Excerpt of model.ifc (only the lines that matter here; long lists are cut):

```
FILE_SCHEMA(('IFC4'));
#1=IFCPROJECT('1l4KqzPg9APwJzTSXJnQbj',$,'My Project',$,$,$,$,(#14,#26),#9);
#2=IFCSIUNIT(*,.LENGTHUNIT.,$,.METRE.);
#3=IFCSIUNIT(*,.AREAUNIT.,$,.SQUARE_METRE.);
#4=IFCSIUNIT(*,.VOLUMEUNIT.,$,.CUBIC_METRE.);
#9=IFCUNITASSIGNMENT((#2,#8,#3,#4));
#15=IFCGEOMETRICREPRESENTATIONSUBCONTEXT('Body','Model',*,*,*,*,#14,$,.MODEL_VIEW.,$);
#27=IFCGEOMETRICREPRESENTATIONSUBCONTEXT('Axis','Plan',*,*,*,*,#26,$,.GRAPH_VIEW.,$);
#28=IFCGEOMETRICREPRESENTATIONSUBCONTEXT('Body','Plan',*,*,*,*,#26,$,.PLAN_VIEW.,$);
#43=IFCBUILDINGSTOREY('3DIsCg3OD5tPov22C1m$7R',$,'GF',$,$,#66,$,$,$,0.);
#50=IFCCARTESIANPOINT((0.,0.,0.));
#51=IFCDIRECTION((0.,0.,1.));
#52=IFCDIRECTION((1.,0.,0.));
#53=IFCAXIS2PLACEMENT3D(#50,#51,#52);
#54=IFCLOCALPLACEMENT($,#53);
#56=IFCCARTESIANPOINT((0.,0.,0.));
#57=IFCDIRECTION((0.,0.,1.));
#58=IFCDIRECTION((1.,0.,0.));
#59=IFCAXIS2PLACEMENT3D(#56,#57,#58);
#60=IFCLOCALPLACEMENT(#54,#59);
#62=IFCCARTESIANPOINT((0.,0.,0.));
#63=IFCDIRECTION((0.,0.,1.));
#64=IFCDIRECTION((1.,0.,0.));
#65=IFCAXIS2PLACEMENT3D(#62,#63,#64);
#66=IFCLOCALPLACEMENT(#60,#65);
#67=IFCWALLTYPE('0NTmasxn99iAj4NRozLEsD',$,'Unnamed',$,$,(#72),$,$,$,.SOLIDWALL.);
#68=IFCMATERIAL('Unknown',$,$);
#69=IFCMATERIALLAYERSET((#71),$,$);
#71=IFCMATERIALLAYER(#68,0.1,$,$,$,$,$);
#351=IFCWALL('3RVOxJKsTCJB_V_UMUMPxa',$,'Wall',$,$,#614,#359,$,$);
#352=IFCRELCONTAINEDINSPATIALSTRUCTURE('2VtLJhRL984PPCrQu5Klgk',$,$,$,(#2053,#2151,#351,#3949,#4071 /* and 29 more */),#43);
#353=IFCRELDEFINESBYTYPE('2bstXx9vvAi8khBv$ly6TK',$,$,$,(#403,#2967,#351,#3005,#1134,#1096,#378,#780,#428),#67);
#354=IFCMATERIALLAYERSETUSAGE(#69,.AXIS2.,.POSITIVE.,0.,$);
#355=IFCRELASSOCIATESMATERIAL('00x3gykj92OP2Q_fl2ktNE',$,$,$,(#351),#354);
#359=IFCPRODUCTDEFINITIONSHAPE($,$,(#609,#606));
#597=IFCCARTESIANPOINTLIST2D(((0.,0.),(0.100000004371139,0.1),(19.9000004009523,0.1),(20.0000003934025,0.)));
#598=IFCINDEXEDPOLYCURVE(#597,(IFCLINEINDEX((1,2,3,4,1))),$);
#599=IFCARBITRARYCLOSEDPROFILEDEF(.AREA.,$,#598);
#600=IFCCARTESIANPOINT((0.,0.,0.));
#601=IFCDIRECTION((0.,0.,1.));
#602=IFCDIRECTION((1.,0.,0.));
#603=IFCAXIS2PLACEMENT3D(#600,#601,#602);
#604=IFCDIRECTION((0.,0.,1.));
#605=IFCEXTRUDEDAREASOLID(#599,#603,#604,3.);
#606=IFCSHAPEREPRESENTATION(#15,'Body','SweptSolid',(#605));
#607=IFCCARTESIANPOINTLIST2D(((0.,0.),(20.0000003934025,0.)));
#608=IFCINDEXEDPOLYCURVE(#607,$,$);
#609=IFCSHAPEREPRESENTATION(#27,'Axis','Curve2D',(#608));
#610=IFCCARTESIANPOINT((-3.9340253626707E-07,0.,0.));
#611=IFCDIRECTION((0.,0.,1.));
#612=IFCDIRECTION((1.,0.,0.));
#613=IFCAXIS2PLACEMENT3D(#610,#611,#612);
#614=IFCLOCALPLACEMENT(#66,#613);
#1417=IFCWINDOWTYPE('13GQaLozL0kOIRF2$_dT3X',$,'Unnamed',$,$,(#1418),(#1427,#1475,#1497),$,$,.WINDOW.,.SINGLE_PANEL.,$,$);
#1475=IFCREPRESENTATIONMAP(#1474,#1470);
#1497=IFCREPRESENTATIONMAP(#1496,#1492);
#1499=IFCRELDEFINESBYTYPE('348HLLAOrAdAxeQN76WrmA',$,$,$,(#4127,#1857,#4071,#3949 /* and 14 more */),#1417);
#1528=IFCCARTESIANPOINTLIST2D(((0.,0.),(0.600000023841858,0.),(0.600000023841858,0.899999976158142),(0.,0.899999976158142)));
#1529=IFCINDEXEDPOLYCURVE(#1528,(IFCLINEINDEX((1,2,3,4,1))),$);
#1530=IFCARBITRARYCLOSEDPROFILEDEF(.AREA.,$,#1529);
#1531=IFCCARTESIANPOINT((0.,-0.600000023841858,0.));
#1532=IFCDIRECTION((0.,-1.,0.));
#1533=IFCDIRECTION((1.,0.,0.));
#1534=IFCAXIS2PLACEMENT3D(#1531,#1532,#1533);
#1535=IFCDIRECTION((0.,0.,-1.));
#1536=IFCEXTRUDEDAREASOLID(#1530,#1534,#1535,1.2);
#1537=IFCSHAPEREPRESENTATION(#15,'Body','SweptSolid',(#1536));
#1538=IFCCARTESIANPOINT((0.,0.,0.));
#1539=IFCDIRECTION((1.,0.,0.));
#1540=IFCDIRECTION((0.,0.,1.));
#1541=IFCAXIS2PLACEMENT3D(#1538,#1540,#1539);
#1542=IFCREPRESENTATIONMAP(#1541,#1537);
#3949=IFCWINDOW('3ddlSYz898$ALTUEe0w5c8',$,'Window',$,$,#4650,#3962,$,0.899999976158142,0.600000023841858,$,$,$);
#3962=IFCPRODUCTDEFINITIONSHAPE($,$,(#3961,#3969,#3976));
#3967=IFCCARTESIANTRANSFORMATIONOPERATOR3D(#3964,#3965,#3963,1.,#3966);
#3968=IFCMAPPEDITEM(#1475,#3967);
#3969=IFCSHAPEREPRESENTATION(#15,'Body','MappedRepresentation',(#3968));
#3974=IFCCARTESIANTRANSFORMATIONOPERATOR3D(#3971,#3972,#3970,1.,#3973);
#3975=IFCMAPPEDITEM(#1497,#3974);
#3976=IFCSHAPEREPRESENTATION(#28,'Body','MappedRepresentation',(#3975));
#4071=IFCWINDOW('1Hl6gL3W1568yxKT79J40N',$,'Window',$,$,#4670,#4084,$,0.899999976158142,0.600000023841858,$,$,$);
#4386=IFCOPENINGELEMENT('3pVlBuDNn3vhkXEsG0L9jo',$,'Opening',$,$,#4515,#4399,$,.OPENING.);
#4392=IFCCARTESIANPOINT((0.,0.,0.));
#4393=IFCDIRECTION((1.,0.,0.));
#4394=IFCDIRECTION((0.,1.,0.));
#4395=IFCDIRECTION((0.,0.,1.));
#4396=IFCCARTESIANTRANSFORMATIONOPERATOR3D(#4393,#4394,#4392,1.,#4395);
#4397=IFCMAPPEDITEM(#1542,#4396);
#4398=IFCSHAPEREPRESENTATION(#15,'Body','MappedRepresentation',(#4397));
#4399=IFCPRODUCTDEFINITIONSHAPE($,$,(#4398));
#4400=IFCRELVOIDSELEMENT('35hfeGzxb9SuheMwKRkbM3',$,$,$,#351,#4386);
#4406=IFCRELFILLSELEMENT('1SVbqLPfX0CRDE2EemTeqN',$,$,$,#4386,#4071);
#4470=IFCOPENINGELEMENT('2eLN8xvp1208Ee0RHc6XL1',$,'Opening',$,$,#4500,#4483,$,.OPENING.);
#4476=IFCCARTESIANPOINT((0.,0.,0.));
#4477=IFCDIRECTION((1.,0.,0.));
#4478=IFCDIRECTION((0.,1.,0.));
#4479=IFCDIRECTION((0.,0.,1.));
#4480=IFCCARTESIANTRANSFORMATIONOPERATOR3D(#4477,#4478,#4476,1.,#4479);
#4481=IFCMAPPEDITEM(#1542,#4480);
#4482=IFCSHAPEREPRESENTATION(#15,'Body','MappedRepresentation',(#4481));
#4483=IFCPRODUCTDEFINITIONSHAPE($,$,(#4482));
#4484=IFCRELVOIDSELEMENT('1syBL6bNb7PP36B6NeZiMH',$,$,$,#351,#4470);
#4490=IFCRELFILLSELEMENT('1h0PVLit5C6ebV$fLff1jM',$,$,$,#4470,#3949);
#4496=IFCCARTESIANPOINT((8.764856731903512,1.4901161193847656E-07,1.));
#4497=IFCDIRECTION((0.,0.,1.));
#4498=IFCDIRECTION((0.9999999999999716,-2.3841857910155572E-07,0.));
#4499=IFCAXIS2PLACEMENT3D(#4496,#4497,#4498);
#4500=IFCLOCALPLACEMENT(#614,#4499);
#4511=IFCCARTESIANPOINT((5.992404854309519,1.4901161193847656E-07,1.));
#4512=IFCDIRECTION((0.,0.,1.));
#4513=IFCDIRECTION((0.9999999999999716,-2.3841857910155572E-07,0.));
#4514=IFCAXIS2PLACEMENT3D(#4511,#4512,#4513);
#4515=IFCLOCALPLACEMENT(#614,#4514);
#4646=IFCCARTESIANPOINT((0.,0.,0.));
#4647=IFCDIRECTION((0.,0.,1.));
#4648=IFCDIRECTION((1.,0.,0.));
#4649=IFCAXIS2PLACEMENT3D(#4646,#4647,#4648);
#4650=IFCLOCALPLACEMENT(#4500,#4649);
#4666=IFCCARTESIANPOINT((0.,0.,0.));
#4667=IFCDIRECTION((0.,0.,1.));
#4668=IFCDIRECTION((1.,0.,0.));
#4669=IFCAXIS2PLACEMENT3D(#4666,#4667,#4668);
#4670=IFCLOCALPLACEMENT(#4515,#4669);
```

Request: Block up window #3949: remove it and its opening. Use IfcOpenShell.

```python
import ifcopenshell
import ifcopenshell.api.feature
import ifcopenshell.api.root
import ifcopenshell.geom
import ifcopenshell.util.shape

model = ifcopenshell.open("model.ifc")
settings = ifcopenshell.geom.settings()


def volume(element):
    """Net volume in cubic metres, openings subtracted."""
    shape = ifcopenshell.geom.create_shape(settings, element)
    return ifcopenshell.util.shape.get_volume(shape.geometry)


window = model.by_guid("3ddlSYz898$ALTUEe0w5c8")
opening = window.FillsVoids[0].RelatingOpeningElement
wall = opening.VoidsElements[0].RelatingBuildingElement
before = volume(wall)

ifcopenshell.api.root.remove_product(model, product=window)
ifcopenshell.api.feature.remove_feature(model, feature=opening)

after = volume(wall)

print(f"wall volume {before:.3f} -> {after:.3f} m3")

model.write("model_rev.ifc")
```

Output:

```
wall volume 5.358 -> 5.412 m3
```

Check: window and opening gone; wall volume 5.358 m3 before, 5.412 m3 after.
